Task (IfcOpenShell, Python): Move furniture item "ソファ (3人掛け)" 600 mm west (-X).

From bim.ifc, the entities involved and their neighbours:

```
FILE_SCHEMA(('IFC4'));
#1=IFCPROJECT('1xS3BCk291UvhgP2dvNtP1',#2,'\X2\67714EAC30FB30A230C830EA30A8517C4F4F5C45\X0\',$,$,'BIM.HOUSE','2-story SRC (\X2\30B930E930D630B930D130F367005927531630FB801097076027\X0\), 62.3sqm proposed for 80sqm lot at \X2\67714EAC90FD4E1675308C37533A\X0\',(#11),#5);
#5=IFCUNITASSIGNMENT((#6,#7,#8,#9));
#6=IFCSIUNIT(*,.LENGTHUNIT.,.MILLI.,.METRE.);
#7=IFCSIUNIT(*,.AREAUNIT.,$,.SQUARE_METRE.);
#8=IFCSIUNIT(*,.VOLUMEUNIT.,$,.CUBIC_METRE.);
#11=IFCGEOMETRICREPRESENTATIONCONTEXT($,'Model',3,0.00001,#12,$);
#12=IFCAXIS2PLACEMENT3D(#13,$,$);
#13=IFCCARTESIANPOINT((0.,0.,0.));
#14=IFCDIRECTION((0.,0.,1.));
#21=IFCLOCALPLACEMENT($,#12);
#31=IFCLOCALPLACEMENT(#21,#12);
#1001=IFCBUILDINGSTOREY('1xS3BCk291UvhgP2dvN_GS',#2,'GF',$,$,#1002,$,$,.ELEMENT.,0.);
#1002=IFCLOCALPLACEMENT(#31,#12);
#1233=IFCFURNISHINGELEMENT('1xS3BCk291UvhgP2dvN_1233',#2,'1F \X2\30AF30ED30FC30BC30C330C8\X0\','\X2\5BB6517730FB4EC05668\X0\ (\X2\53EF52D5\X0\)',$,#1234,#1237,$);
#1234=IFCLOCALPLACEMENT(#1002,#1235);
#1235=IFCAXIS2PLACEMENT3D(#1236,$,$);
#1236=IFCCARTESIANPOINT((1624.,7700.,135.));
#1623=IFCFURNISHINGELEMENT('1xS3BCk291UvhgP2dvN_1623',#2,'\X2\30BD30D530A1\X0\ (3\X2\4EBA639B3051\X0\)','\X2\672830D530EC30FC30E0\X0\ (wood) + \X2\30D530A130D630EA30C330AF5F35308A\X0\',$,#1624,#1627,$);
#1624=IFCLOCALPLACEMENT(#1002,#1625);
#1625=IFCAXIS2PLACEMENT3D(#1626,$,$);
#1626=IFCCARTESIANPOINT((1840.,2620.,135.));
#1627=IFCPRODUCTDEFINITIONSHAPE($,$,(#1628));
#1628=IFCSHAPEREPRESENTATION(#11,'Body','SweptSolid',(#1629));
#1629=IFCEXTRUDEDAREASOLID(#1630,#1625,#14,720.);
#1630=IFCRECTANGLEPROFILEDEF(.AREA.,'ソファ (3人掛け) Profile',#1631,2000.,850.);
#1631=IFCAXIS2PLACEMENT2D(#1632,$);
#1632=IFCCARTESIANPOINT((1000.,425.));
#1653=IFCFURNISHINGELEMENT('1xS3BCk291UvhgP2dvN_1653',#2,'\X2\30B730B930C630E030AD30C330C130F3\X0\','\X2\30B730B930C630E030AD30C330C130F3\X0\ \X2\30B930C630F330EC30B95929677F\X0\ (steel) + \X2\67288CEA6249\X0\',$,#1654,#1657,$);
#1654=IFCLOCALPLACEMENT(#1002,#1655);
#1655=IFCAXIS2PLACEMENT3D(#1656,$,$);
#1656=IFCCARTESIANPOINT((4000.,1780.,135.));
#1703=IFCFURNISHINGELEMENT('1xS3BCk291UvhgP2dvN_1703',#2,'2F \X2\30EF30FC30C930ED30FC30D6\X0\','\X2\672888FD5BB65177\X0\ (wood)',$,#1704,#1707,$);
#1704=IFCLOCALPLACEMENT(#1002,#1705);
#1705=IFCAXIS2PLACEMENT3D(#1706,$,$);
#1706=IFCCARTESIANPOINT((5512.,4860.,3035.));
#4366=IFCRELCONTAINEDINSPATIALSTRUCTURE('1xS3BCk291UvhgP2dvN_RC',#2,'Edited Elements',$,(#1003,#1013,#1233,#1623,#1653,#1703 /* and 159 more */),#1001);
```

```python
import ifcopenshell
import ifcopenshell.api.geometry
import ifcopenshell.util.placement
import ifcopenshell.util.unit

model = ifcopenshell.open("bim.ifc")
unit_scale = ifcopenshell.util.unit.calculate_unit_scale(model)

item = model.by_guid("1xS3BCk291UvhgP2dvN_1623")
matrix = ifcopenshell.util.placement.get_local_placement(item.ObjectPlacement)
matrix[0, 3] -= 0.6 / unit_scale
ifcopenshell.api.geometry.edit_object_placement(model, product=item, matrix=matrix, is_si=False)

print(ifcopenshell.util.placement.get_local_placement(item.ObjectPlacement).round(3) + 0.0)

model.write("bim-out.ifc")
```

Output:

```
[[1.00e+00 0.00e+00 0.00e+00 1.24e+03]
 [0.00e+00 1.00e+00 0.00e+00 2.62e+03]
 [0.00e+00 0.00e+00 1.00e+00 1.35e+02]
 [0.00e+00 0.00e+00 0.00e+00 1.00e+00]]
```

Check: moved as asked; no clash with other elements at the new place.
